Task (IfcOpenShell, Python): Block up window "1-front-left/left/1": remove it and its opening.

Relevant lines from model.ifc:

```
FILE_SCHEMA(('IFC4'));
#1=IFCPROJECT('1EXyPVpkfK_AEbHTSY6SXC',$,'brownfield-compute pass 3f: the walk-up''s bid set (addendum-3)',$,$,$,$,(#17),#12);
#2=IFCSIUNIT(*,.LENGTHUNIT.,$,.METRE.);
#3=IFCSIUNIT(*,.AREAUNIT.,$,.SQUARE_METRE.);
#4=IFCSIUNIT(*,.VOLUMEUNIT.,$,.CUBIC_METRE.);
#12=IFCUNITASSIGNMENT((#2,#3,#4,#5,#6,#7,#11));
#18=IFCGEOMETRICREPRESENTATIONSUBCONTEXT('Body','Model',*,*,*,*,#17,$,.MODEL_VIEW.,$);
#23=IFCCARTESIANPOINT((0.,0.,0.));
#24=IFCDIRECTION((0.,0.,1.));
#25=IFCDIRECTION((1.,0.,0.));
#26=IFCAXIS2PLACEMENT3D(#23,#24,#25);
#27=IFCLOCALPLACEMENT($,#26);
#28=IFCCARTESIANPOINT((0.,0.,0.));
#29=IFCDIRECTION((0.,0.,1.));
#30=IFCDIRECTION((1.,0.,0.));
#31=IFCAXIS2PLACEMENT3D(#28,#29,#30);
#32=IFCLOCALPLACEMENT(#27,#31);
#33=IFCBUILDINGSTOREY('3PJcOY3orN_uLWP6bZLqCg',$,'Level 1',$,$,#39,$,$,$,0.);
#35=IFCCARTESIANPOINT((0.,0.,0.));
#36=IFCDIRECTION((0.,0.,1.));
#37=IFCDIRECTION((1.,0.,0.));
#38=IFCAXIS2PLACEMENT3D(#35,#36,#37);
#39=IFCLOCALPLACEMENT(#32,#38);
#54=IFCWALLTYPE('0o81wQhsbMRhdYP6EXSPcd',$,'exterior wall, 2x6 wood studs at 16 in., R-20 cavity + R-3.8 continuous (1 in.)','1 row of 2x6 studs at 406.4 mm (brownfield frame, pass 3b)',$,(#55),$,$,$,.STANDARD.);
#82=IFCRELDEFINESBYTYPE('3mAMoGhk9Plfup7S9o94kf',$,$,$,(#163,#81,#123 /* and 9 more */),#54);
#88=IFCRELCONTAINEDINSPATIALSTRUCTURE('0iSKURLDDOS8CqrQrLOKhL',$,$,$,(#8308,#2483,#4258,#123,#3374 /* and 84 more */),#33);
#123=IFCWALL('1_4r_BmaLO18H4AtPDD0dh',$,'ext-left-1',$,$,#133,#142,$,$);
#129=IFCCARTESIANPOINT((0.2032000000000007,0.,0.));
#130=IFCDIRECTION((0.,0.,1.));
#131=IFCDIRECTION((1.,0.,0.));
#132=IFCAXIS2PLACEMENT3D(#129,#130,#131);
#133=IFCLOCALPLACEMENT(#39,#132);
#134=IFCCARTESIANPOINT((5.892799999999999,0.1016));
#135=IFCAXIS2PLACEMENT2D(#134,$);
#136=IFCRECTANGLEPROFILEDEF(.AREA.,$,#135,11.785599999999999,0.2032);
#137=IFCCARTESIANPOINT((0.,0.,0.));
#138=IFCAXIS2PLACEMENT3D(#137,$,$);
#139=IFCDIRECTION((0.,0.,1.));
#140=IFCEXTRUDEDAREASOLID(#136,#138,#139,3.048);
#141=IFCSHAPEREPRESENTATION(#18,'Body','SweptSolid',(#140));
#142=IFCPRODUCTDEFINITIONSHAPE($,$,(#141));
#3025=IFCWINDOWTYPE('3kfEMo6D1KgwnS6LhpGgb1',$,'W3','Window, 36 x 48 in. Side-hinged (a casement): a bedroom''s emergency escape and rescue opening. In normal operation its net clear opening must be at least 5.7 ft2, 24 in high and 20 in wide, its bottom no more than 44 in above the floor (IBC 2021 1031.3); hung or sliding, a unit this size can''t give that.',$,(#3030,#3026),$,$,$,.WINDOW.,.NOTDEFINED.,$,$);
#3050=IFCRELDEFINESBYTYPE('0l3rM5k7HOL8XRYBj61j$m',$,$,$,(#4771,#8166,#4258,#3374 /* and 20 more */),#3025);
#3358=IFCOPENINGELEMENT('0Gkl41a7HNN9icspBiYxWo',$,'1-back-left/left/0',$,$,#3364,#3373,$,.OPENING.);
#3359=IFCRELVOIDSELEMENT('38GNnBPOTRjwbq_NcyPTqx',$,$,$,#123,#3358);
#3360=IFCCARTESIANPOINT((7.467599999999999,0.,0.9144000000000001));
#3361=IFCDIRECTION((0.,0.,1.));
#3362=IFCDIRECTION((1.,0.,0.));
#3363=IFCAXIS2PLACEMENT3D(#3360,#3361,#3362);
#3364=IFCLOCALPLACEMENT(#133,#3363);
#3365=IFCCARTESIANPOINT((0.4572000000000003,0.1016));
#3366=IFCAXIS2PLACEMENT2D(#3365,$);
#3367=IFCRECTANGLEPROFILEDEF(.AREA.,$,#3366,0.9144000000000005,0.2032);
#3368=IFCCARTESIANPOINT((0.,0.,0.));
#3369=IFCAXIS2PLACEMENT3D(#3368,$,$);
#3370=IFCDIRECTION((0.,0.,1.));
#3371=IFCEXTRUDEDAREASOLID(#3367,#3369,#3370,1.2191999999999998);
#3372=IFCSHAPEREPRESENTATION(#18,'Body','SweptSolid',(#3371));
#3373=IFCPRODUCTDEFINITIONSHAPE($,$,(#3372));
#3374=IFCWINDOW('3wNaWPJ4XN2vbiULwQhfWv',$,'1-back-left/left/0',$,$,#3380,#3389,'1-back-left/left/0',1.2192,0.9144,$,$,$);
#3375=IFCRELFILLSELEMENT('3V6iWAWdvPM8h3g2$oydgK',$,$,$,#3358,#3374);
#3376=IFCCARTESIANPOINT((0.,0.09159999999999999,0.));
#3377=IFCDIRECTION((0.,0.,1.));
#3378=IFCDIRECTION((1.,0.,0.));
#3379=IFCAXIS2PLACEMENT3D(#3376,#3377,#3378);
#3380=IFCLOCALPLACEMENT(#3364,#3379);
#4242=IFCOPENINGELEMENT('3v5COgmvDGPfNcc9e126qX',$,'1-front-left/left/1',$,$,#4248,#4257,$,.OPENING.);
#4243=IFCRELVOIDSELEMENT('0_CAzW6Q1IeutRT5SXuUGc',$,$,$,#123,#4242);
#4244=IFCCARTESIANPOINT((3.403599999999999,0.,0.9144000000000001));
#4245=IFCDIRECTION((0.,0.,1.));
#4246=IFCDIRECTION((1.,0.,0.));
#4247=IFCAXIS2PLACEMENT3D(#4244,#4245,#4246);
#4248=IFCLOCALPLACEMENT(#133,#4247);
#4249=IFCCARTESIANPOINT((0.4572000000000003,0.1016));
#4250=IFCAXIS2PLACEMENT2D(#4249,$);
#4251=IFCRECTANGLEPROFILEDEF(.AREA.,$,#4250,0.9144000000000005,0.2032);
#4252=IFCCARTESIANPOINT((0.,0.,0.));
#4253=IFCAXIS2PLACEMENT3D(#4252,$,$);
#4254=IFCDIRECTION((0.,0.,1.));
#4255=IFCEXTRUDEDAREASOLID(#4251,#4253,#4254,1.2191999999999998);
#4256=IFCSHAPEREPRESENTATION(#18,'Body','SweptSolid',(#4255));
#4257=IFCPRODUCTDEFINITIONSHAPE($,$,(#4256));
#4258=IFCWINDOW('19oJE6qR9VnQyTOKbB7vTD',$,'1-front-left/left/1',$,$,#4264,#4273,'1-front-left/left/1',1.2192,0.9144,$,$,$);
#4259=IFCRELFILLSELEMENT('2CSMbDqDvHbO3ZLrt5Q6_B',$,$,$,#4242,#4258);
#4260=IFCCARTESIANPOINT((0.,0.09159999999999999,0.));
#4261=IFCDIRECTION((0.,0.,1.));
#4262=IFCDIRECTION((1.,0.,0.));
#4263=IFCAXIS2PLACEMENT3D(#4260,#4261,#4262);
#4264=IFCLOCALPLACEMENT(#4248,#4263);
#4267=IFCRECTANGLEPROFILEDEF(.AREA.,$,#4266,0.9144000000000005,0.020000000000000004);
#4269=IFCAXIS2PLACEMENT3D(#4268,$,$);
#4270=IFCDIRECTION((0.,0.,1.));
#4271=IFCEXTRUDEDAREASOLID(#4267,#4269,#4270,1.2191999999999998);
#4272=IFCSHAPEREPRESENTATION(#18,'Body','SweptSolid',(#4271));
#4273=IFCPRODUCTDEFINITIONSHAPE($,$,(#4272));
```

```python
import ifcopenshell
import ifcopenshell.api.feature
import ifcopenshell.api.root
import ifcopenshell.geom
import ifcopenshell.util.shape

model = ifcopenshell.open("model.ifc")
settings = ifcopenshell.geom.settings()


def volume(element):
    """Net volume in cubic metres, openings subtracted."""
    shape = ifcopenshell.geom.create_shape(settings, element)
    return ifcopenshell.util.shape.get_volume(shape.geometry)


window = model.by_guid("19oJE6qR9VnQyTOKbB7vTD")
opening = window.FillsVoids[0].RelatingOpeningElement
wall = opening.VoidsElements[0].RelatingBuildingElement
before = volume(wall)

ifcopenshell.api.root.remove_product(model, product=window)
ifcopenshell.api.feature.remove_feature(model, feature=opening)

after = volume(wall)

print(f"wall volume {before:.3f} -> {after:.3f} m3")

model.write("model-out.ifc")
```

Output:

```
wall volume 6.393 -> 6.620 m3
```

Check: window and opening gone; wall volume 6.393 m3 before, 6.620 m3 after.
